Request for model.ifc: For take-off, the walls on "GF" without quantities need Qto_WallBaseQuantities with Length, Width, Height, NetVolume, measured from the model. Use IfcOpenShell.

First a look at what the model holds.

```python
import ifcopenshell
import ifcopenshell.util.element
import ifcopenshell.util.unit

model = ifcopenshell.open("model.ifc")
print(model.schema)
for unit_type in ("LENGTHUNIT", "AREAUNIT", "VOLUMEUNIT"):
    print(unit_type, ifcopenshell.util.unit.calculate_unit_scale(model, unit_type))
storey = next(s for s in model.by_type("IfcBuildingStorey") if s.Name == "GF")
walls = [e for e in ifcopenshell.util.element.get_decomposition(storey) if e.is_a("IfcWall")]
for e in sorted(walls, key=lambda e: e.id()):
    print(e.id(), e.is_a(), e.Name, list(ifcopenshell.util.element.get_psets(e, qtos_only=True)), sep=" | ")
```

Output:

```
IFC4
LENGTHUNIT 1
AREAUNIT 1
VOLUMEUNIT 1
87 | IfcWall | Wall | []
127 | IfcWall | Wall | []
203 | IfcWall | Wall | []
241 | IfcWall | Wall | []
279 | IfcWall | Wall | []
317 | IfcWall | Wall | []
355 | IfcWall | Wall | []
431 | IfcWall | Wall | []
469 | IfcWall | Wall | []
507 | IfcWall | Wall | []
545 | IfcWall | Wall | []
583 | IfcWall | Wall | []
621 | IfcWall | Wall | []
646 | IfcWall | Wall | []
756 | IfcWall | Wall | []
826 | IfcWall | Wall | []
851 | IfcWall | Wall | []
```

```python
import ifcopenshell
import ifcopenshell.api.pset
import ifcopenshell.geom
import ifcopenshell.util.element
import ifcopenshell.util.shape
import ifcopenshell.util.unit

model = ifcopenshell.open("model.ifc")
unit_scale = ifcopenshell.util.unit.calculate_unit_scale(model)
volume_scale = ifcopenshell.util.unit.calculate_unit_scale(model, "VOLUMEUNIT")
settings = ifcopenshell.geom.settings()

storey = next(s for s in model.by_type("IfcBuildingStorey") if s.Name == "GF")
walls = [e for e in ifcopenshell.util.element.get_decomposition(storey) if e.is_a("IfcWall")]

for e in sorted(walls, key=lambda e: e.id()):
    if ifcopenshell.util.element.get_psets(e, qtos_only=True, should_inherit=False):
        continue
    # Geometry comes back in metres, in the element's own axes.
    shape = ifcopenshell.geom.create_shape(settings, e)
    values = {
        "Length": ifcopenshell.util.shape.get_x(shape.geometry) / unit_scale,
        "Width": ifcopenshell.util.shape.get_y(shape.geometry) / unit_scale,
        "Height": ifcopenshell.util.shape.get_z(shape.geometry) / unit_scale,
        "NetVolume": ifcopenshell.util.shape.get_volume(shape.geometry) / volume_scale,
    }
    qto = ifcopenshell.api.pset.add_qto(model, product=e, name="Qto_WallBaseQuantities")
    ifcopenshell.api.pset.edit_qto(model, qto=qto, properties=values)
    print(e.id(), {k: round(v, 3) for k, v in values.items()})

model.write("model_rev.ifc")
```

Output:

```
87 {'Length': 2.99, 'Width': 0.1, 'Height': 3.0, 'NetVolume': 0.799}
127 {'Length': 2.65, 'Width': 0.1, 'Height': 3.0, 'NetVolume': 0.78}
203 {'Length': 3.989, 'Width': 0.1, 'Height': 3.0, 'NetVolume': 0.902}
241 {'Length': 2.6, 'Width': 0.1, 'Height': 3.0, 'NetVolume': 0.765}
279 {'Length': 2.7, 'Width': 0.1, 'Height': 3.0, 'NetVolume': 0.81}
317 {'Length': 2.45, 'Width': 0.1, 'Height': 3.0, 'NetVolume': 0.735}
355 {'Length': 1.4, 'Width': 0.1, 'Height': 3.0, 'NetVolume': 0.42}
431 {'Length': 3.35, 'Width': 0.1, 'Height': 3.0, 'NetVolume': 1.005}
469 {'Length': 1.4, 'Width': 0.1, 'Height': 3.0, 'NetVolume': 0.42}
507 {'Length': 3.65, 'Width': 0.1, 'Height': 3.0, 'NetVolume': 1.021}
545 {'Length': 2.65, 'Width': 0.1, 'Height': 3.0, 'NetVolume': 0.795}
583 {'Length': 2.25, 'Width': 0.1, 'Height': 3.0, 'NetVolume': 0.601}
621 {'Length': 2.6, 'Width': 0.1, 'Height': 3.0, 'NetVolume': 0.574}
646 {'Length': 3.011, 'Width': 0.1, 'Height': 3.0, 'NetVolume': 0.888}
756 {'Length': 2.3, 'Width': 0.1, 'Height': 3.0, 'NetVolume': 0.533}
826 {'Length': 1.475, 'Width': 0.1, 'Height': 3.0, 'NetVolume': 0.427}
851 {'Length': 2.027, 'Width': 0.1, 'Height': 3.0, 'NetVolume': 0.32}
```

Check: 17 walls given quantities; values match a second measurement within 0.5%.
